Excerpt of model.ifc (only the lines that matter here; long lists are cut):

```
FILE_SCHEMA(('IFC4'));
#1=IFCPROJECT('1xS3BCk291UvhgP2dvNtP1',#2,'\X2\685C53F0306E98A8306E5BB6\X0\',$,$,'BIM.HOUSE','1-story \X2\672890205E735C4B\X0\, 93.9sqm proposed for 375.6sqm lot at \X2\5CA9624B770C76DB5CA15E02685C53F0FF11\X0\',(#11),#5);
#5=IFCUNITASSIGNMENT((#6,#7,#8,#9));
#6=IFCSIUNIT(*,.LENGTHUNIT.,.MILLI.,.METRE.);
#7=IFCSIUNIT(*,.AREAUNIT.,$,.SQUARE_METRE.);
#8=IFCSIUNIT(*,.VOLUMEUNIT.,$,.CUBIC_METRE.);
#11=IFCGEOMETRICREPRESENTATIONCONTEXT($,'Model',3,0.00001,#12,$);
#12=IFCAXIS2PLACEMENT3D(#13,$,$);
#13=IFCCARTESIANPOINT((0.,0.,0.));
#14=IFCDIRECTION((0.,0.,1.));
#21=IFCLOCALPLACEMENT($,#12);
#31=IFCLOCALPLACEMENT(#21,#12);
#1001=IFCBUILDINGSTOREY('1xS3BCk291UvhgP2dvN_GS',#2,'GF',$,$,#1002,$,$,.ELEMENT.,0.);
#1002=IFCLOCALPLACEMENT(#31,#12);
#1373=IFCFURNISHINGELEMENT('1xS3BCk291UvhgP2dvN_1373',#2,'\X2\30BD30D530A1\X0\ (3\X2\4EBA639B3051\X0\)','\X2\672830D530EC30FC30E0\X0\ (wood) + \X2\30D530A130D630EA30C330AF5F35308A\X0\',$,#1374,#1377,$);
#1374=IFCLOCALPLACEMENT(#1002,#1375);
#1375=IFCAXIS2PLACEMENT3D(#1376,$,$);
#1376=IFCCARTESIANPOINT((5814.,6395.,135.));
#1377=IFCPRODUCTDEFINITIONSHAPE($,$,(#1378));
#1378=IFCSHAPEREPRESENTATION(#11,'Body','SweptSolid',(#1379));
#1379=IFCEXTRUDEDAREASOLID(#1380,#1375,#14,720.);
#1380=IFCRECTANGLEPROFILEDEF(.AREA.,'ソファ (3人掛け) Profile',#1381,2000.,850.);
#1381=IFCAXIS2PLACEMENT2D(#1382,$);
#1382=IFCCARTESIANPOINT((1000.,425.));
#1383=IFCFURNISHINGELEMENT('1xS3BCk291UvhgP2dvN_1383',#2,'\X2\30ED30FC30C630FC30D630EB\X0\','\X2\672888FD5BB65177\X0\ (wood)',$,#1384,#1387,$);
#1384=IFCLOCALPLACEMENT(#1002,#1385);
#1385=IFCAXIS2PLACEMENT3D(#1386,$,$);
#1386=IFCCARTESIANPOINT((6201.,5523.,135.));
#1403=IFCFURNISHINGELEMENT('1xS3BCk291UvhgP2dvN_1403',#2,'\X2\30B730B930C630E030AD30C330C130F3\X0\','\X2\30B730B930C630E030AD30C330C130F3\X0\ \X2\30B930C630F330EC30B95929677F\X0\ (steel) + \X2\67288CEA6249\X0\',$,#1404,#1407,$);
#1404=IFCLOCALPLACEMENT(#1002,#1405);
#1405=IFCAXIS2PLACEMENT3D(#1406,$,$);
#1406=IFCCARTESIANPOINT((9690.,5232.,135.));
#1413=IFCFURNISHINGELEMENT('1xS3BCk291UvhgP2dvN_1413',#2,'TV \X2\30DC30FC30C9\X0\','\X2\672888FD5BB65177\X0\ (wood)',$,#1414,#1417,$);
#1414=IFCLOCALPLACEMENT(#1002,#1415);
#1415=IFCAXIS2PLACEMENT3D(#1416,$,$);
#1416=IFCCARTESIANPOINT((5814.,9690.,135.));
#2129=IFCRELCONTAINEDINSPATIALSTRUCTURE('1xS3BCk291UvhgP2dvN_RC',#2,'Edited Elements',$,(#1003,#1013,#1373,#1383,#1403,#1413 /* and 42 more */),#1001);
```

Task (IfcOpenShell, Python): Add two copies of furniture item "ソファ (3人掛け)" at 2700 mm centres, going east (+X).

```python
import numpy as np
import ifcopenshell
import ifcopenshell.api.geometry
import ifcopenshell.api.root
import ifcopenshell.util.element
import ifcopenshell.util.placement

model = ifcopenshell.open("model.ifc")


def reuse_history(source, copy):
    """copy_class also copies each property set's owner history, people and application; keep the originals."""
    for rel in copy.IsDefinedBy:
        if rel.is_a("IfcRelDefinesByProperties") and (history := rel.RelatingPropertyDefinition.OwnerHistory):
            rel.RelatingPropertyDefinition.OwnerHistory = source.OwnerHistory
            ifcopenshell.util.element.remove_deep2(model, history)


source = model.by_id(1373)
base = ifcopenshell.util.placement.get_local_placement(source.ObjectPlacement)
step = np.array([1.0, 0.0, 0.0]) * 2700.0

for i in range(1, 3):
    copy = ifcopenshell.api.root.copy_class(model, product=source)
    copy.Representation = ifcopenshell.util.element.copy_deep(
        model, source.Representation, exclude=["IfcGeometricRepresentationContext", "IfcRepresentationMap"]
    )
    reuse_history(source, copy)
    matrix = base.copy()
    matrix[:3, 3] += i * step
    print("added at", matrix[:3, 3].round(3) + 0.0)
    ifcopenshell.api.geometry.edit_object_placement(model, product=copy, matrix=matrix, is_si=False)

model.write("model-out.ifc")
```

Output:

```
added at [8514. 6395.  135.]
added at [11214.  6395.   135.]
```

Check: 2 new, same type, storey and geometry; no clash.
